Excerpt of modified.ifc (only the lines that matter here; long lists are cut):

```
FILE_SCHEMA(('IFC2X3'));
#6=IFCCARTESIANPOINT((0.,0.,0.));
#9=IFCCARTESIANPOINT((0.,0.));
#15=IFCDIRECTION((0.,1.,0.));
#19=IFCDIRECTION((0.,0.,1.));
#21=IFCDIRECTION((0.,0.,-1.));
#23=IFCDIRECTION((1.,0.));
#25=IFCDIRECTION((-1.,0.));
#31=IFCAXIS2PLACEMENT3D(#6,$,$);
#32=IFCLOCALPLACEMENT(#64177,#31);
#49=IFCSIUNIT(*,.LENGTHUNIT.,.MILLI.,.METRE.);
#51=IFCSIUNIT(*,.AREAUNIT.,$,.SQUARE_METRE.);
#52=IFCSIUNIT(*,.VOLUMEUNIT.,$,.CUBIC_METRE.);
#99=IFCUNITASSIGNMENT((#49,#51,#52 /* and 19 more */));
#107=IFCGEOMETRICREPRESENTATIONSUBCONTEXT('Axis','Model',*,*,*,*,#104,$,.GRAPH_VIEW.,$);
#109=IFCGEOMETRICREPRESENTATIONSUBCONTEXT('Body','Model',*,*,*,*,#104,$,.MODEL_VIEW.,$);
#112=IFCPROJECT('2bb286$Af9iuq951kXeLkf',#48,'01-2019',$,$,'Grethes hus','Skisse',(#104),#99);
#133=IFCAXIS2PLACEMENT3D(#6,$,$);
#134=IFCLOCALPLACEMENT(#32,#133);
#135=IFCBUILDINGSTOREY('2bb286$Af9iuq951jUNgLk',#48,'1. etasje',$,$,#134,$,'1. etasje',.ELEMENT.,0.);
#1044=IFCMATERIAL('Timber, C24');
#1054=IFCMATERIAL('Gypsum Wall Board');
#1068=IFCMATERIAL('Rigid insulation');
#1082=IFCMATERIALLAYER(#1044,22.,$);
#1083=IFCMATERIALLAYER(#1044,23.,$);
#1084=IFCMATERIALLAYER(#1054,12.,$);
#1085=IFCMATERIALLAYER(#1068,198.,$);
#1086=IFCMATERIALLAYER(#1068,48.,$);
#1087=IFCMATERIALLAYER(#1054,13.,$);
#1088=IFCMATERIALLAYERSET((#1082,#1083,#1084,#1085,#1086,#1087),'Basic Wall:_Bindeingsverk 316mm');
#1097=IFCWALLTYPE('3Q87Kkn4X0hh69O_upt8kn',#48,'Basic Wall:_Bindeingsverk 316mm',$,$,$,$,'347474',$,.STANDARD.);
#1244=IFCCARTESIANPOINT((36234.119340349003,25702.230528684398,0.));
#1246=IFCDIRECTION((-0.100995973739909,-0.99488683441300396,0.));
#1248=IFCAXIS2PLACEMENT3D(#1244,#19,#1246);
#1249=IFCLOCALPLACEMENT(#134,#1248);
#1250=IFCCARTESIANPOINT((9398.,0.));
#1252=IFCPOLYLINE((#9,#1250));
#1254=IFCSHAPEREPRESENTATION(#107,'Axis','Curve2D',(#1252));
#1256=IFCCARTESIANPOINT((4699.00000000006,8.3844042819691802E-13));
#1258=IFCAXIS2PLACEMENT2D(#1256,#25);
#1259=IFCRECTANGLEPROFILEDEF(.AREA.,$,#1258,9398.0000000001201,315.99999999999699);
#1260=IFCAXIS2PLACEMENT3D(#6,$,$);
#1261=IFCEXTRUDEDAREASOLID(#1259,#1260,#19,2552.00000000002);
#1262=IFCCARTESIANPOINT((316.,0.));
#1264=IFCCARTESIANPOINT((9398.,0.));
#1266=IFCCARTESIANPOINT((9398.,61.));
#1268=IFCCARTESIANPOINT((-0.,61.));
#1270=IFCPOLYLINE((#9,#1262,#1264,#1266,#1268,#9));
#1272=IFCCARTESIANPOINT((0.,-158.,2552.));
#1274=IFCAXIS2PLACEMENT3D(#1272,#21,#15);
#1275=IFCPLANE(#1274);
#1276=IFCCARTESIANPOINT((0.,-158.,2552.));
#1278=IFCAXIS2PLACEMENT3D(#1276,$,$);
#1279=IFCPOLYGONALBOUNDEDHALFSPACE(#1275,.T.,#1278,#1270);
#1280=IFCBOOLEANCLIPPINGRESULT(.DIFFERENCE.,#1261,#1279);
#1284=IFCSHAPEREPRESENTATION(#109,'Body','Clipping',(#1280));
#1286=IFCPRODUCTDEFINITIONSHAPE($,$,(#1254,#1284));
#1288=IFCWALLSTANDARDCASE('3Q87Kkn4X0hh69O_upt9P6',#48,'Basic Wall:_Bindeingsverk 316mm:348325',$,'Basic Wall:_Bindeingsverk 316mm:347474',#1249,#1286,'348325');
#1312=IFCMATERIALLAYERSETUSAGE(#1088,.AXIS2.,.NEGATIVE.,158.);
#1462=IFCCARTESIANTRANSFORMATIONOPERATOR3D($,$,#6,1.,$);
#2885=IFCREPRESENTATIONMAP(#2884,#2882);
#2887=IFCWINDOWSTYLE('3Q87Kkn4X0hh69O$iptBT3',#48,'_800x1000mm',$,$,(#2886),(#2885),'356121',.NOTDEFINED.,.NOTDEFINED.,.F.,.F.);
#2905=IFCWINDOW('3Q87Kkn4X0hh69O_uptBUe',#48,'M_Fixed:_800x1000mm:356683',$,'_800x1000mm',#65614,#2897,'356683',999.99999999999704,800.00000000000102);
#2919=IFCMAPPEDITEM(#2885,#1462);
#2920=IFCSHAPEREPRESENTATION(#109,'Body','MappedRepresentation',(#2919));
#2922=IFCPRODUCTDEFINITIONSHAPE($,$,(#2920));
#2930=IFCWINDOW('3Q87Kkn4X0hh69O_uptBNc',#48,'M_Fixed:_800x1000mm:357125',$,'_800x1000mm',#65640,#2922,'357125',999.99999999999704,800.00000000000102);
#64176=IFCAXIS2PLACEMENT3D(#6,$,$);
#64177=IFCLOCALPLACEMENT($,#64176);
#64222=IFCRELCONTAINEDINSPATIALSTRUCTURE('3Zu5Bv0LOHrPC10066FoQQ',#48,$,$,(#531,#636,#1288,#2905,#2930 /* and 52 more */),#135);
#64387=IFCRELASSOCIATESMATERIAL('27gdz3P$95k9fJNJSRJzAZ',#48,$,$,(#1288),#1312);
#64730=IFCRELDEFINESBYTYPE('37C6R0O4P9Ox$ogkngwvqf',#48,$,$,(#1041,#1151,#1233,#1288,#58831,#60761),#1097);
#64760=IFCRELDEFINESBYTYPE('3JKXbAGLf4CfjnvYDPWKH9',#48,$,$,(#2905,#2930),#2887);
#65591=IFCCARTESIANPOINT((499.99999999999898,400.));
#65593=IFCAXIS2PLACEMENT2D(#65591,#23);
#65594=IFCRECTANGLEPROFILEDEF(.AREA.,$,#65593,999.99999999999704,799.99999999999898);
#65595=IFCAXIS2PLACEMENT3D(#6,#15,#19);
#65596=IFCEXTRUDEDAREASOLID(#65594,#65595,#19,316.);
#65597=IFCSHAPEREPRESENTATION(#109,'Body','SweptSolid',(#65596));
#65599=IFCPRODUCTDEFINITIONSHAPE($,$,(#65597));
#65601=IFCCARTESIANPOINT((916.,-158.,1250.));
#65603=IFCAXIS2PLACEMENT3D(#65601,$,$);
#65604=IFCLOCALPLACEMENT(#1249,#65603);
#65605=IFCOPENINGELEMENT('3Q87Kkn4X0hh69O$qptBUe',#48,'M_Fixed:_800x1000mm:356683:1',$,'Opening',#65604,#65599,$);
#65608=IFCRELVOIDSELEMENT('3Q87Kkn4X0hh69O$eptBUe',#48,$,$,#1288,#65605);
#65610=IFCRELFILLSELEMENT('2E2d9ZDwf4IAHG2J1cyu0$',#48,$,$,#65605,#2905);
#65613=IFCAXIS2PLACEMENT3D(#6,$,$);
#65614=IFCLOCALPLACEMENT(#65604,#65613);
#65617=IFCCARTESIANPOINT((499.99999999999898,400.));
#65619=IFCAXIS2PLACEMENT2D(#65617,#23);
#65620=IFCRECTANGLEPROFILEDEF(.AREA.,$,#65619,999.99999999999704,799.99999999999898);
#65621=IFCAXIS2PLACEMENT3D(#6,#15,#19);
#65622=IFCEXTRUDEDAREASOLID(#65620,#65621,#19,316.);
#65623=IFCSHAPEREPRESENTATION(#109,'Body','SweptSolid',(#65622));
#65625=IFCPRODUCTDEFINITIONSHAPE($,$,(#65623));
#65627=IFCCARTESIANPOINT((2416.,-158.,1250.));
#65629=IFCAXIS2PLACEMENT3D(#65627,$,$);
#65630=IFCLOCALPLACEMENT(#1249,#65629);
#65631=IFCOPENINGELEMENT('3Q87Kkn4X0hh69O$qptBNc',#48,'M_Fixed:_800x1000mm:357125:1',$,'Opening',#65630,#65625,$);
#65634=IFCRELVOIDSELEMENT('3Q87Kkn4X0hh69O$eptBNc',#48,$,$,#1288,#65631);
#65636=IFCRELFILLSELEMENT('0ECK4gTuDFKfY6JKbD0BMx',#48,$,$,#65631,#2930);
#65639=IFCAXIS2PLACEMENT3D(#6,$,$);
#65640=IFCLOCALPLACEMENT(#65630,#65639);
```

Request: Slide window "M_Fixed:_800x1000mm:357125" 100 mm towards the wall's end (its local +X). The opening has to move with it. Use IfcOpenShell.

```python
import ifcopenshell
import ifcopenshell.api.geometry
import ifcopenshell.util.placement

model = ifcopenshell.open("modified.ifc")

window = model.by_guid("3Q87Kkn4X0hh69O_uptBNc")
opening = window.FillsVoids[0].RelatingOpeningElement
wall = opening.VoidsElements[0].RelatingBuildingElement

wall_matrix = ifcopenshell.util.placement.get_local_placement(wall.ObjectPlacement)
shift = wall_matrix[:3, 0] * 100.0
before = ifcopenshell.util.placement.get_local_placement(window.ObjectPlacement)[:3, 3].copy()

# The window is placed relative to its opening, so it follows when the opening moves.
matrix = ifcopenshell.util.placement.get_local_placement(opening.ObjectPlacement)
matrix[:3, 3] += shift
ifcopenshell.api.geometry.edit_object_placement(
    model, product=opening, matrix=matrix, is_si=False, should_transform_children=True
)

after = ifcopenshell.util.placement.get_local_placement(window.ObjectPlacement)[:3, 3]
print("window moved by", (after - before).round(3) + 0.0)

model.write("modified_updated.ifc")
```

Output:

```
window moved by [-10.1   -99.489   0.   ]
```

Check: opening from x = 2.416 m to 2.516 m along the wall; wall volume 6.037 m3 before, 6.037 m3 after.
